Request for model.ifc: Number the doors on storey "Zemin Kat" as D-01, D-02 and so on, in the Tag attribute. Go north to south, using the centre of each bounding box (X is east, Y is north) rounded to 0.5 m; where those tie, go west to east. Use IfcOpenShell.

First a look at what the model holds.

```python
import ifcopenshell
import ifcopenshell.util.element
import ifcopenshell.util.placement

model = ifcopenshell.open("model.ifc")
print(model.schema)
storey = next(s for s in model.by_type("IfcBuildingStorey") if s.Name == "Zemin Kat")
doors = [e for e in ifcopenshell.util.element.get_decomposition(storey) if e.is_a("IfcDoor")]
for e in sorted(doors, key=lambda e: e.id()):
    origin = ifcopenshell.util.placement.get_local_placement(e.ObjectPlacement)[:3, 3]
    print(e.id(), e.Tag, e.Name, origin.round(2) + 0.0, sep=" | ")
```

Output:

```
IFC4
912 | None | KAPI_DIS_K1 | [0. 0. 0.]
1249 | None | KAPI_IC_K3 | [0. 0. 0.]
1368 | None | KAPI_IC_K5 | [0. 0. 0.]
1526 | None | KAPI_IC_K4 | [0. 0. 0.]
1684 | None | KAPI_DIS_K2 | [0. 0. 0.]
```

```python
import ifcopenshell
import ifcopenshell.geom
import ifcopenshell.util.element
import ifcopenshell.util.shape

model = ifcopenshell.open("model.ifc")
settings = ifcopenshell.geom.settings()
settings.set("use-world-coords", True)


def centre(element):
    shape = ifcopenshell.geom.create_shape(settings, element)
    return ifcopenshell.util.shape.get_bbox_centroid(shape.geometry)


storey = next(s for s in model.by_type("IfcBuildingStorey") if s.Name == "Zemin Kat")
doors = [e for e in ifcopenshell.util.element.get_decomposition(storey) if e.is_a("IfcDoor")]

# Insertion points can sit at a corner or the storey origin, so sort by the geometry (in metres).
centres = {e: centre(e) for e in doors}
doors.sort(key=lambda e: (-round(centres[e][1] / 0.5), centres[e][0]))

for i, e in enumerate(doors, start=1):
    number = f"D-{i:02d}"
    e.Tag = number
    print(e.id(), number)

model.write("model-out.ifc")
```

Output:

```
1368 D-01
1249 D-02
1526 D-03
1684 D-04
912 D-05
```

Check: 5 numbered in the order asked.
